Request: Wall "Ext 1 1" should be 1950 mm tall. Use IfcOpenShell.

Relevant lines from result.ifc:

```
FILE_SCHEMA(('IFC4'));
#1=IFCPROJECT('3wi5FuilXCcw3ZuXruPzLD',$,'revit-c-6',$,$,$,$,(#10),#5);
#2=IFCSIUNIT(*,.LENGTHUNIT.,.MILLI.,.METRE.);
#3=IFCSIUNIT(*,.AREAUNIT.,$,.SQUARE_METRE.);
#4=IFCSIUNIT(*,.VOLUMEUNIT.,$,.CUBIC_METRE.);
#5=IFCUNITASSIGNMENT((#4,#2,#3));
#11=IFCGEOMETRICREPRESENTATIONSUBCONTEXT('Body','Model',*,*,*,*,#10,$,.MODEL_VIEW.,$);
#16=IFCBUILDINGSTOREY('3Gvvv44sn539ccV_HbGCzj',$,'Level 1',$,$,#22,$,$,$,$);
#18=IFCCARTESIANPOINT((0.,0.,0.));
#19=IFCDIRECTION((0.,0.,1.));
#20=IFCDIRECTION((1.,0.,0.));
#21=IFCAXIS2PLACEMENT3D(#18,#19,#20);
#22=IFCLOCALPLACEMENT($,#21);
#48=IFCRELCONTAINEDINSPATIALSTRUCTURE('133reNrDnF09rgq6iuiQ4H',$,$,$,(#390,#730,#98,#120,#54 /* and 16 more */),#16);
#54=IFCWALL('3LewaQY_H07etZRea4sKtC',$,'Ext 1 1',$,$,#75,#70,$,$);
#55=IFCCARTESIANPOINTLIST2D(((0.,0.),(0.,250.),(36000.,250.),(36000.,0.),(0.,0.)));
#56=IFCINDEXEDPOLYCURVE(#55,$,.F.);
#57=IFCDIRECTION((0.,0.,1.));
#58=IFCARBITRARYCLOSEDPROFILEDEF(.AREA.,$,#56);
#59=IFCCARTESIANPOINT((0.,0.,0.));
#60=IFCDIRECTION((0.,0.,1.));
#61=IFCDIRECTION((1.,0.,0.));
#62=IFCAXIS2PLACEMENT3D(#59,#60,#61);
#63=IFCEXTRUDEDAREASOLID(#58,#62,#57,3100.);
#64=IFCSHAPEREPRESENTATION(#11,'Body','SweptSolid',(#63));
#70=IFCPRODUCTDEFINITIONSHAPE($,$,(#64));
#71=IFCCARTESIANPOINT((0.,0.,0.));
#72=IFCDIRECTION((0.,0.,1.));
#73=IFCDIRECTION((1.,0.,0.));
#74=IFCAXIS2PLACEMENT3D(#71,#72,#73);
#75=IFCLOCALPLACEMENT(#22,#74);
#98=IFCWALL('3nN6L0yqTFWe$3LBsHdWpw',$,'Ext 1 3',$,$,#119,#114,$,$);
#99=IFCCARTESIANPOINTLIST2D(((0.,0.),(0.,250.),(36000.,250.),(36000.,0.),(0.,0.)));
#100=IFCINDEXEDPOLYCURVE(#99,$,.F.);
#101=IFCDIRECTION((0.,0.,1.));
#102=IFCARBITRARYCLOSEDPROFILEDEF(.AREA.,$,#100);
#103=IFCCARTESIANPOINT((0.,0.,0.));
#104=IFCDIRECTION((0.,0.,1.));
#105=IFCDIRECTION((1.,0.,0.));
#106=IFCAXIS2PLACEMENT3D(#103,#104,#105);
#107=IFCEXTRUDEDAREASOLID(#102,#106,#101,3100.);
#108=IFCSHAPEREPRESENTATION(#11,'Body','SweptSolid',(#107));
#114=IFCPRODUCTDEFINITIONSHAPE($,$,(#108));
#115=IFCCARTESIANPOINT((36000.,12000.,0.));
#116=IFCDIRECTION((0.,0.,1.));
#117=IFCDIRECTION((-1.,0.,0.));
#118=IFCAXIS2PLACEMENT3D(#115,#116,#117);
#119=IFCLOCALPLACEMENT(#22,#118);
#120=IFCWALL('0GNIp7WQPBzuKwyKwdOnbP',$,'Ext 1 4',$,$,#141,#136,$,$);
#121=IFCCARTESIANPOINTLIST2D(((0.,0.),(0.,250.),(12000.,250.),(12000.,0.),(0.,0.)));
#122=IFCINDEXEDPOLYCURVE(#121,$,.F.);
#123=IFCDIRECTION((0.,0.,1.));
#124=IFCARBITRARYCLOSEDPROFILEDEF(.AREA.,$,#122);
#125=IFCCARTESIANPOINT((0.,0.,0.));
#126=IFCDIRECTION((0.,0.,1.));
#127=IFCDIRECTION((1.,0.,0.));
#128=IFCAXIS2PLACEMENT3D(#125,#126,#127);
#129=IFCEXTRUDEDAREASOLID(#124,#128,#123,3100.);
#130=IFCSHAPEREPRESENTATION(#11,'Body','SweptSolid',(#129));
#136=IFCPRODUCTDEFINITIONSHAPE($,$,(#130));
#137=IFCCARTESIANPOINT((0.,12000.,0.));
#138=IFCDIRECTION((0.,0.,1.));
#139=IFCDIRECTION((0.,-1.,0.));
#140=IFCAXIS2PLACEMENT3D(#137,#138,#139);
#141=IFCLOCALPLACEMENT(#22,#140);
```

```python
import ifcopenshell
import ifcopenshell.geom
import ifcopenshell.util.representation
import ifcopenshell.util.shape

model = ifcopenshell.open("result.ifc")
settings = ifcopenshell.geom.settings()


def volume(element):
    """Net volume in cubic metres, openings subtracted."""
    shape = ifcopenshell.geom.create_shape(settings, element)
    return ifcopenshell.util.shape.get_volume(shape.geometry)


wall = model.by_guid("3LewaQY_H07etZRea4sKtC")
before = volume(wall)

body = ifcopenshell.util.representation.get_representation(wall, "Model", "Body")
solid = body.Items[0]
old_height = solid.Depth
solid.Depth = 1950.0
after = volume(wall)

print(f"height {old_height:g} -> {solid.Depth:g}, volume {before:.3f} -> {after:.3f} m3")

model.write("result-out.ifc")
```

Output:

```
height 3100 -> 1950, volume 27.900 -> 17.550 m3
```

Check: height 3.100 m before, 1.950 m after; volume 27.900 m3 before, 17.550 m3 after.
